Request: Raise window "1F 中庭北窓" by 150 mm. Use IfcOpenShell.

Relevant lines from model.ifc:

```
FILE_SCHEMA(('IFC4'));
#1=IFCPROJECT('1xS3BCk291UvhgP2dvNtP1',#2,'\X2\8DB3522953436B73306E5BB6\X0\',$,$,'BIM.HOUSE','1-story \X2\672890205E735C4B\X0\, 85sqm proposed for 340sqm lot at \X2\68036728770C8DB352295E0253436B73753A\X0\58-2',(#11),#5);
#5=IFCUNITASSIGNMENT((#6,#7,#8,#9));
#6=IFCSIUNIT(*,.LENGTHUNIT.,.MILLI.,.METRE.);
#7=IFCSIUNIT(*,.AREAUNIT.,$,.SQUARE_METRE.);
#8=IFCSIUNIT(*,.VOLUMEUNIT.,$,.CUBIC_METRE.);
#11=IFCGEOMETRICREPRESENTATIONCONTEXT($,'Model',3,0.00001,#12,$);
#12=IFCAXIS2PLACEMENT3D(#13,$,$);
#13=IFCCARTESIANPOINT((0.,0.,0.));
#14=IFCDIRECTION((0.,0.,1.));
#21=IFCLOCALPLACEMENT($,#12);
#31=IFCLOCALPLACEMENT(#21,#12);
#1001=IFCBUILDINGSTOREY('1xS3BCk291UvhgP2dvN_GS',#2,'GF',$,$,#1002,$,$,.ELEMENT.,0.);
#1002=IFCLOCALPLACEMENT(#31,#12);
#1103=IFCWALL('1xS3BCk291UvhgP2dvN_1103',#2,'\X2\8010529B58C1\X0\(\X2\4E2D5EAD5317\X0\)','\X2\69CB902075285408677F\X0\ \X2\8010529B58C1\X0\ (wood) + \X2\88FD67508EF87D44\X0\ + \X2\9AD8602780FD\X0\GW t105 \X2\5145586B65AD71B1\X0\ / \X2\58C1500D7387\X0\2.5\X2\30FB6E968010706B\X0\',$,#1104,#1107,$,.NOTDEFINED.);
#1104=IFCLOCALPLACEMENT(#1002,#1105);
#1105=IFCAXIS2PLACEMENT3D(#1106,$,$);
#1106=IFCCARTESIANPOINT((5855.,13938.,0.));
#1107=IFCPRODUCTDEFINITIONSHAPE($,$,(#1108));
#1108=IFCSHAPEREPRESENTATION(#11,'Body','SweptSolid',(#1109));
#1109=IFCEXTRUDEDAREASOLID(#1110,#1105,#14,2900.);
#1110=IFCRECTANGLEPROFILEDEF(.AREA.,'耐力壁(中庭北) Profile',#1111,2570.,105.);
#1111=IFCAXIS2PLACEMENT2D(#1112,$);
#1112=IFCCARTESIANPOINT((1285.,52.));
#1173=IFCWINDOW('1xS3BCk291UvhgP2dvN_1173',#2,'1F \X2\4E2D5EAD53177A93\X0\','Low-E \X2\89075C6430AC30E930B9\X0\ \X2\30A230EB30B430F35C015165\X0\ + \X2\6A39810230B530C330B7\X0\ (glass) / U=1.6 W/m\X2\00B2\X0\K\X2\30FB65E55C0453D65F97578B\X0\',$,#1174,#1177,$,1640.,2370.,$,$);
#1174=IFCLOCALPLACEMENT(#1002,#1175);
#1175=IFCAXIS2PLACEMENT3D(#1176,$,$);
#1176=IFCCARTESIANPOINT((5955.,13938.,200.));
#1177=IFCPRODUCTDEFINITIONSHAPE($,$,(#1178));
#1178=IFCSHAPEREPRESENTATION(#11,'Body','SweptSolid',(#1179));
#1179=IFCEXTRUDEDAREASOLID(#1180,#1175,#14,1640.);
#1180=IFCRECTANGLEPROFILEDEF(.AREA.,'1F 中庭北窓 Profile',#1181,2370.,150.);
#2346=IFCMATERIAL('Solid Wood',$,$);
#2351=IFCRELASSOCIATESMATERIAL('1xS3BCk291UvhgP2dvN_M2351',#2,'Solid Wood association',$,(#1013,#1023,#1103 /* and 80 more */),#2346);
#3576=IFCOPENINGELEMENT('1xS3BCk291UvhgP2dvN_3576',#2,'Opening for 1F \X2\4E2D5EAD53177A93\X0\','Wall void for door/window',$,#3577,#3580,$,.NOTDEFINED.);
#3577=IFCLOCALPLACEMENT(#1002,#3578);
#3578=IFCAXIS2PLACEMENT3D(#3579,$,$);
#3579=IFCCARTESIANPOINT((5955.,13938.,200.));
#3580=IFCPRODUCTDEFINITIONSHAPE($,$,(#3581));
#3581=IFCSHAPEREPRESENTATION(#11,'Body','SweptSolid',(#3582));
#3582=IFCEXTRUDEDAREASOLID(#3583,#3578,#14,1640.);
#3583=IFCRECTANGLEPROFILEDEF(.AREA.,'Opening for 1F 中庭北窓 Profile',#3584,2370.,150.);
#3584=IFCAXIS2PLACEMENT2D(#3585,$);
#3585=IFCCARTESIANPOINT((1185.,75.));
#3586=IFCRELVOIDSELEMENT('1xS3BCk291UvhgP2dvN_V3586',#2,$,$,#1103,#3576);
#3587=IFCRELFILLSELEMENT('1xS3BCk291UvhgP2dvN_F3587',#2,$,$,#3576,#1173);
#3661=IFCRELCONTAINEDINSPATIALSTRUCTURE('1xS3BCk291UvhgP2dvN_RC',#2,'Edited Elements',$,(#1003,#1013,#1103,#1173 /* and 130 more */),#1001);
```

```python
import numpy as np
import ifcopenshell
import ifcopenshell.api.geometry
import ifcopenshell.util.placement
import ifcopenshell.util.unit

model = ifcopenshell.open("model.ifc")
unit_scale = ifcopenshell.util.unit.calculate_unit_scale(model)

window = model.by_guid("1xS3BCk291UvhgP2dvN_1173")
opening = window.FillsVoids[0].RelatingOpeningElement
dz = 150.0

shift = np.array([0.0, 0.0, dz])
# The window is not placed relative to its opening, so move both.
for product in (opening, window):
    matrix = ifcopenshell.util.placement.get_local_placement(product.ObjectPlacement)
    matrix[:3, 3] += shift
    ifcopenshell.api.geometry.edit_object_placement(model, product=product, matrix=matrix, is_si=False)

print(f"moved by {dz * unit_scale:+.3f} m")

model.write("model_edited.ifc")
```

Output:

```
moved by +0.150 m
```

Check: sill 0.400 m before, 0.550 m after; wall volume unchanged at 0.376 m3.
